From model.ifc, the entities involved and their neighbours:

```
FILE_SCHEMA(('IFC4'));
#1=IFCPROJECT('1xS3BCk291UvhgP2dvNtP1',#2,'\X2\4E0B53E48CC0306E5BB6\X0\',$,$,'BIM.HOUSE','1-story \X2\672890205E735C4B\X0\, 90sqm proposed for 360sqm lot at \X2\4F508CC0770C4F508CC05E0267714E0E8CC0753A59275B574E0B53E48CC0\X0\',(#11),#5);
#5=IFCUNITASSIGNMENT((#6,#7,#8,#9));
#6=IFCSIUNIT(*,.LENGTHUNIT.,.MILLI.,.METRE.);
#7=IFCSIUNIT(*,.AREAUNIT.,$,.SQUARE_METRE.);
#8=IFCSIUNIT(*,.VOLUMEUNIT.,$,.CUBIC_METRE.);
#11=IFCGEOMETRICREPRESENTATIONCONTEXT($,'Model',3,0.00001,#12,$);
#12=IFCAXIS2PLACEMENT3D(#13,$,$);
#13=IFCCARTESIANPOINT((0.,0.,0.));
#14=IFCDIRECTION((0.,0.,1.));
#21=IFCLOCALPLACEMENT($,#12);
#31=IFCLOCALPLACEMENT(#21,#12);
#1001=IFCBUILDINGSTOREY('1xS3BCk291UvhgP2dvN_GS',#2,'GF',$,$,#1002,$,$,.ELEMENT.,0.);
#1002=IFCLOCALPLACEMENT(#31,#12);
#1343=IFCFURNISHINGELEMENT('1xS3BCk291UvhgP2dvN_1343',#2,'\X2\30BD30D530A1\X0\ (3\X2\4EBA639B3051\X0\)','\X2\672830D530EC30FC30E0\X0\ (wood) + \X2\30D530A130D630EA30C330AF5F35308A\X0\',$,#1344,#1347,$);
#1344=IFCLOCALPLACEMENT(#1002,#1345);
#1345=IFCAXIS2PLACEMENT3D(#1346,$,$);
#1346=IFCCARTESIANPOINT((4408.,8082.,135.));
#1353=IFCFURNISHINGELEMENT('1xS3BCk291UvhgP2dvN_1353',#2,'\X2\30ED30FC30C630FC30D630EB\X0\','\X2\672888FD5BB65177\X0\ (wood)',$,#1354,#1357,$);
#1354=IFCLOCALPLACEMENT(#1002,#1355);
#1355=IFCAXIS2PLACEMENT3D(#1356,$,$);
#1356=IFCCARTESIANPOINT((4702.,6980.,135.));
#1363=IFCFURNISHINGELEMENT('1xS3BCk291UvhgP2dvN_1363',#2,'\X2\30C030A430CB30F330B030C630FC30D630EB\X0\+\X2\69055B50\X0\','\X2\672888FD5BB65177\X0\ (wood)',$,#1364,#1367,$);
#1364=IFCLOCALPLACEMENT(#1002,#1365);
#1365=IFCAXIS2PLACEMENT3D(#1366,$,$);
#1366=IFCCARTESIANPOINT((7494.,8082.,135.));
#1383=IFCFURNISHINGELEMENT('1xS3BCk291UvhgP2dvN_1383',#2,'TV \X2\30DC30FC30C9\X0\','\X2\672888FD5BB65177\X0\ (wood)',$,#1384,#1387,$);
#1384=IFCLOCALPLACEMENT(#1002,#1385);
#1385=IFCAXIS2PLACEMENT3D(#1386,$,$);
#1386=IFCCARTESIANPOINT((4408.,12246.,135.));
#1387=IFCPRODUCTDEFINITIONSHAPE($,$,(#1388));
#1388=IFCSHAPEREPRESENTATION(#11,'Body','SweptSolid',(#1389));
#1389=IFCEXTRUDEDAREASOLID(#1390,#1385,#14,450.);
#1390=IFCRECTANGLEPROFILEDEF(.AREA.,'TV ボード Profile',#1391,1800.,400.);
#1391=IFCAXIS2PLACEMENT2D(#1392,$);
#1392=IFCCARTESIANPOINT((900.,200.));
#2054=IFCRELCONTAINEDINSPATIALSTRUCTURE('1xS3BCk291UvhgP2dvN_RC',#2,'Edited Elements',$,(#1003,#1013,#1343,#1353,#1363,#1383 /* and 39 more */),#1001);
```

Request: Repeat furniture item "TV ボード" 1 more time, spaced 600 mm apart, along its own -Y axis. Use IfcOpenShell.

```python
import ifcopenshell
import ifcopenshell.api.geometry
import ifcopenshell.api.root
import ifcopenshell.util.element
import ifcopenshell.util.placement

model = ifcopenshell.open("model.ifc")


def reuse_history(source, copy):
    """copy_class also copies each property set's owner history, people and application; keep the originals."""
    for rel in copy.IsDefinedBy:
        if rel.is_a("IfcRelDefinesByProperties") and (history := rel.RelatingPropertyDefinition.OwnerHistory):
            rel.RelatingPropertyDefinition.OwnerHistory = source.OwnerHistory
            ifcopenshell.util.element.remove_deep2(model, history)


source = model.by_guid("1xS3BCk291UvhgP2dvN_1383")
base = ifcopenshell.util.placement.get_local_placement(source.ObjectPlacement)
step = -base[:3, 1] * 600.0

for i in range(1, 2):
    copy = ifcopenshell.api.root.copy_class(model, product=source)
    copy.Representation = ifcopenshell.util.element.copy_deep(
        model, source.Representation, exclude=["IfcGeometricRepresentationContext", "IfcRepresentationMap"]
    )
    reuse_history(source, copy)
    matrix = base.copy()
    matrix[:3, 3] += i * step
    print("added at", matrix[:3, 3].round(3) + 0.0)
    ifcopenshell.api.geometry.edit_object_placement(model, product=copy, matrix=matrix, is_si=False)

model.write("model_updated.ifc")
```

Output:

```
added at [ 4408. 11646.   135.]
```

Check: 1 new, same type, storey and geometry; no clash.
